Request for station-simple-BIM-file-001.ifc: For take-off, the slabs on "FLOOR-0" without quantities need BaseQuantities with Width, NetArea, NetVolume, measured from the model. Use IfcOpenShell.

First a look at what the model holds.

```python
import ifcopenshell
import ifcopenshell.util.element
import ifcopenshell.util.unit

model = ifcopenshell.open("station-simple-BIM-file-001.ifc")
print(model.schema)
for unit_type in ("LENGTHUNIT", "AREAUNIT", "VOLUMEUNIT"):
    print(unit_type, ifcopenshell.util.unit.calculate_unit_scale(model, unit_type))
storey = next(s for s in model.by_type("IfcBuildingStorey") if s.Name == "FLOOR-0")
slabs = [e for e in ifcopenshell.util.element.get_decomposition(storey) if e.is_a("IfcSlab")]
for e in sorted(slabs, key=lambda e: e.id()):
    print(e.id(), e.is_a(), e.Name, list(ifcopenshell.util.element.get_psets(e, qtos_only=True)), sep=" | ")
```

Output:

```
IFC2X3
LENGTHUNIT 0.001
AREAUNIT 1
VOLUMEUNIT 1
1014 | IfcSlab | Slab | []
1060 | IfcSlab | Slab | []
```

```python
import ifcopenshell
import ifcopenshell.api.pset
import ifcopenshell.geom
import ifcopenshell.util.element
import ifcopenshell.util.shape
import ifcopenshell.util.unit

model = ifcopenshell.open("station-simple-BIM-file-001.ifc")
unit_scale = ifcopenshell.util.unit.calculate_unit_scale(model)
area_scale = ifcopenshell.util.unit.calculate_unit_scale(model, "AREAUNIT")
volume_scale = ifcopenshell.util.unit.calculate_unit_scale(model, "VOLUMEUNIT")
settings = ifcopenshell.geom.settings()

storey = next(s for s in model.by_type("IfcBuildingStorey") if s.Name == "FLOOR-0")
slabs = [e for e in ifcopenshell.util.element.get_decomposition(storey) if e.is_a("IfcSlab")]

for e in sorted(slabs, key=lambda e: e.id()):
    if ifcopenshell.util.element.get_psets(e, qtos_only=True, should_inherit=False):
        continue
    # Geometry comes back in metres, in the element's own axes.
    shape = ifcopenshell.geom.create_shape(settings, e)
    values = {
        "Width": ifcopenshell.util.shape.get_z(shape.geometry) / unit_scale,
        "NetArea": ifcopenshell.util.shape.get_footprint_area(shape.geometry) / area_scale,
        "NetVolume": ifcopenshell.util.shape.get_volume(shape.geometry) / volume_scale,
    }
    qto = ifcopenshell.api.pset.add_qto(model, product=e, name="BaseQuantities")
    ifcopenshell.api.pset.edit_qto(model, qto=qto, properties=values)
    print(e.id(), {k: round(v, 3) for k, v in values.items()})

model.write("station-simple-BIM-file-001_v2.ifc")
```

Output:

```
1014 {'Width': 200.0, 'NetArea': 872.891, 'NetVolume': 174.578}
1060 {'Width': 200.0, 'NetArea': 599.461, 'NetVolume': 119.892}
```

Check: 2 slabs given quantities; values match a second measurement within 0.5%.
